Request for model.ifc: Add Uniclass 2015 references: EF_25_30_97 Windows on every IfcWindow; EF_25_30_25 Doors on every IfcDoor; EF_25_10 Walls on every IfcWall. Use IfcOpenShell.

First a look at what the model holds.

```python
import ifcopenshell

model = ifcopenshell.open("model.ifc")
print(model.schema)
print("classifications:", [c.Name for c in model.by_type("IfcClassification")])
for ifc_class in ("IfcDoor", "IfcRoof", "IfcStair", "IfcWall", "IfcWindow"):
    print(ifc_class, len(model.by_type(ifc_class)))
```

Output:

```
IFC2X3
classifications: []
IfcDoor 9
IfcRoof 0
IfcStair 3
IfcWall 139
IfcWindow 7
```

```python
import ifcopenshell
import ifcopenshell.api.classification

model = ifcopenshell.open("model.ifc")

# IFC2X3 requires Source and Edition and has no link from the project to the system.
system = model.create_entity("IfcClassification", Source="NBS", Edition="2015", Name="Uniclass 2015")

codes = {
    "IfcWindow": ("EF_25_30_97", "Windows"),
    "IfcDoor": ("EF_25_30_25", "Doors"),
    "IfcWall": ("EF_25_10", "Walls"),
}
for ifc_class, (code, name) in codes.items():
    products = model.by_type(ifc_class)
    ifcopenshell.api.classification.add_reference(
        model, products=products, classification=system, identification=code, name=name
    )
    print(code, len(products))

model.write("model_edited.ifc")
```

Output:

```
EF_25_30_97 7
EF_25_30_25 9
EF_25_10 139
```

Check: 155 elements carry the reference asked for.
